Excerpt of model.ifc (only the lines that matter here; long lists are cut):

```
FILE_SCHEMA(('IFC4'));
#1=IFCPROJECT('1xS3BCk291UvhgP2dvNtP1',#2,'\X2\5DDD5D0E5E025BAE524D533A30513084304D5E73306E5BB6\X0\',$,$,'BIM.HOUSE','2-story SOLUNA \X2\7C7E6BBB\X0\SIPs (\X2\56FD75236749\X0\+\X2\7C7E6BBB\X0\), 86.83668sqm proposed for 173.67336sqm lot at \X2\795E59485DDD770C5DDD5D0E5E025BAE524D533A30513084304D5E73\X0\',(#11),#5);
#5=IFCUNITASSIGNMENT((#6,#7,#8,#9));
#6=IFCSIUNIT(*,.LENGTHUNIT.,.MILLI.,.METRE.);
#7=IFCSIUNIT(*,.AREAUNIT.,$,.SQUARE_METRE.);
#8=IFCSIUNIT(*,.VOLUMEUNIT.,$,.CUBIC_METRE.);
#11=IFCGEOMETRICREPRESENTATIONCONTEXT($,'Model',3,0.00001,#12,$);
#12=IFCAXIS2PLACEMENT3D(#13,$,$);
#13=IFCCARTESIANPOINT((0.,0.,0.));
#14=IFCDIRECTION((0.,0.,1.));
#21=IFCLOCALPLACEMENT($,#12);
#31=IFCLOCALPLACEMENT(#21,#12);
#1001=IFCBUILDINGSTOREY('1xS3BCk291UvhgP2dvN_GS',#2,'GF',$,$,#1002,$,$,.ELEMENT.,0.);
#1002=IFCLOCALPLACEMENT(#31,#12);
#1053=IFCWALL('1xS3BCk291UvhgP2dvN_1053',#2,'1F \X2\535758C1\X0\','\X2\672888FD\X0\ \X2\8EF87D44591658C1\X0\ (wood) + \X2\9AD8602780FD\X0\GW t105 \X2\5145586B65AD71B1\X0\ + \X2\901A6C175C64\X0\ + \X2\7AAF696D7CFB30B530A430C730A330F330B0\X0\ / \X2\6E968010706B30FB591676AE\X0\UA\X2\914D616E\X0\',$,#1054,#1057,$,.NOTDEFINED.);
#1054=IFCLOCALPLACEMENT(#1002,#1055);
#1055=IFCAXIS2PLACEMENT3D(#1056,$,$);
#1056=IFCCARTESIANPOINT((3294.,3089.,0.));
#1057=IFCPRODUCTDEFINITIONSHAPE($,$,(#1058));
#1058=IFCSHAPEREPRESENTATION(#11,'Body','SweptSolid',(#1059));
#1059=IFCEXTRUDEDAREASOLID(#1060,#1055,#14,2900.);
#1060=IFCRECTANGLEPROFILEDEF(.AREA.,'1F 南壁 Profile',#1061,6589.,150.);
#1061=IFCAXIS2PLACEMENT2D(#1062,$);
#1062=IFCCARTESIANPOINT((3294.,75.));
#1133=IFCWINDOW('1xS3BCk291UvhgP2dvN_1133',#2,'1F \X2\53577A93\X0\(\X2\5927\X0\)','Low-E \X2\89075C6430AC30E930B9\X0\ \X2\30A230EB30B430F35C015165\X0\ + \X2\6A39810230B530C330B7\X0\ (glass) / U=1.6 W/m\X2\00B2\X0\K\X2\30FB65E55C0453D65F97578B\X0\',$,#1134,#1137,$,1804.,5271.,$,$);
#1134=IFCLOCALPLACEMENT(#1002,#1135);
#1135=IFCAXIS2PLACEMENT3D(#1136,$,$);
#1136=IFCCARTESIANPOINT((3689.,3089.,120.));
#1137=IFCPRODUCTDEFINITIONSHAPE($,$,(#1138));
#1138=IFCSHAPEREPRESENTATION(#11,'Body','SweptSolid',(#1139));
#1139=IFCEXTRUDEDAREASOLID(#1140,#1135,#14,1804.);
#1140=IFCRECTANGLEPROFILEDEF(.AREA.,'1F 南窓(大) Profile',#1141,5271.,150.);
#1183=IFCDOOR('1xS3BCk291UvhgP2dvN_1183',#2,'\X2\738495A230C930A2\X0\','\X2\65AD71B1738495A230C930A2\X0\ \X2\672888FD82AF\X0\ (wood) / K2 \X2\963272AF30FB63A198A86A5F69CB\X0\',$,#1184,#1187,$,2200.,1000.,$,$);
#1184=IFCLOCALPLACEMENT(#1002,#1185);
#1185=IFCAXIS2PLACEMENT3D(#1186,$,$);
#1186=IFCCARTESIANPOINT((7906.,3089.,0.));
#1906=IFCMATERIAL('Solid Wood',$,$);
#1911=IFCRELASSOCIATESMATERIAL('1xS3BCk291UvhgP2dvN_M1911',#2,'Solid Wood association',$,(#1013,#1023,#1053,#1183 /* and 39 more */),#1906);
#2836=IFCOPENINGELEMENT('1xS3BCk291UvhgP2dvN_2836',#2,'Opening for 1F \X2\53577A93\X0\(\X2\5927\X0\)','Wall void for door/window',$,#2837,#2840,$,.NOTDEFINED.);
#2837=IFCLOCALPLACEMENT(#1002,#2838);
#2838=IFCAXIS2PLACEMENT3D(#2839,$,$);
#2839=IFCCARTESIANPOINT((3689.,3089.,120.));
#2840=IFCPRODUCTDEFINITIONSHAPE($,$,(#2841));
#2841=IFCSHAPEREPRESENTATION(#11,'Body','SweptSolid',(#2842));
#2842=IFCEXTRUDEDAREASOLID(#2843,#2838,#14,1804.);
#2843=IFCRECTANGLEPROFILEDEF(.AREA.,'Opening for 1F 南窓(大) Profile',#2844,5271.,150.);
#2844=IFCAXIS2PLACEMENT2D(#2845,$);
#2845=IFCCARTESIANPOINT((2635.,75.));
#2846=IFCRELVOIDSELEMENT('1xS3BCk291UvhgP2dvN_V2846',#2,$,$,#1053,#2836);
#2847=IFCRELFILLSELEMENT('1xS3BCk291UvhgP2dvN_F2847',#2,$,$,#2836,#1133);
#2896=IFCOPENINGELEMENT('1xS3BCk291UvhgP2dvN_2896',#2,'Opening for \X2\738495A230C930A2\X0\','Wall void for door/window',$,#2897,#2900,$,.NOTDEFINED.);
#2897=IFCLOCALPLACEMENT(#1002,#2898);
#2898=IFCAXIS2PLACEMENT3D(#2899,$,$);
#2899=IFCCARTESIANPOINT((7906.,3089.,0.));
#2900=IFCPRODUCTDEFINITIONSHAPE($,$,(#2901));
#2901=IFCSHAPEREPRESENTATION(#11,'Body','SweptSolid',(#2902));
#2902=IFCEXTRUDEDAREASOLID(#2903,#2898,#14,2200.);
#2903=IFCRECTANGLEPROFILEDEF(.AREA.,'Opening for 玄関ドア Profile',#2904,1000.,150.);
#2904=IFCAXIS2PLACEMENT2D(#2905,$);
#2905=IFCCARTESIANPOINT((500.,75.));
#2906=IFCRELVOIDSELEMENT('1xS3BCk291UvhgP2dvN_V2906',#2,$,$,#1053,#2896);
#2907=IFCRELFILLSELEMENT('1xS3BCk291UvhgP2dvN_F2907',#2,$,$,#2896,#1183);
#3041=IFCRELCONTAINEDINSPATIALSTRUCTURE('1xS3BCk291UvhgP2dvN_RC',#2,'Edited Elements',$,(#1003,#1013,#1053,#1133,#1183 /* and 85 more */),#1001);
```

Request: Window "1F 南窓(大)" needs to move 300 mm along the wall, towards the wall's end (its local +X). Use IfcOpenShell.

```python
import ifcopenshell
import ifcopenshell.api.geometry
import ifcopenshell.util.placement
import ifcopenshell.util.unit

model = ifcopenshell.open("model.ifc")
unit_scale = ifcopenshell.util.unit.calculate_unit_scale(model)

window = model.by_id(1133)
opening = window.FillsVoids[0].RelatingOpeningElement
wall = opening.VoidsElements[0].RelatingBuildingElement

wall_matrix = ifcopenshell.util.placement.get_local_placement(wall.ObjectPlacement)
shift = wall_matrix[:3, 0] * 0.3 / unit_scale
before = ifcopenshell.util.placement.get_local_placement(window.ObjectPlacement)[:3, 3].copy()

# The window is not placed relative to its opening, so move both.
for product in (opening, window):
    matrix = ifcopenshell.util.placement.get_local_placement(product.ObjectPlacement)
    matrix[:3, 3] += shift
    ifcopenshell.api.geometry.edit_object_placement(model, product=product, matrix=matrix, is_si=False)

after = ifcopenshell.util.placement.get_local_placement(window.ObjectPlacement)[:3, 3]
print("window moved by", (after - before).round(3) + 0.0)

model.write("model_updated.ifc")
```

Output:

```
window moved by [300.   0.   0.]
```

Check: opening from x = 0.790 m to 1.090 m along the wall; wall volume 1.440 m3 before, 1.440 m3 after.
